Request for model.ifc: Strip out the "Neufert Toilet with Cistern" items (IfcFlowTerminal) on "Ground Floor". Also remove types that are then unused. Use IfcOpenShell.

First a look at what the model holds.

```python
import ifcopenshell
import ifcopenshell.util.element

model = ifcopenshell.open("model.ifc")
print(model.schema)
storey = next(s for s in model.by_type("IfcBuildingStorey") if s.Name == "Ground Floor")
terminals = [e for e in ifcopenshell.util.element.get_decomposition(storey) if e.is_a("IfcFlowTerminal")]
seen = {}
for e in terminals:
    element_type = ifcopenshell.util.element.get_type(e)
    name = element_type.Name if element_type not in (None, e) else None
    seen[name] = seen.get(name, 0) + 1
for name, count in sorted(seen.items(), key=str):
    print(count, "x", name)
```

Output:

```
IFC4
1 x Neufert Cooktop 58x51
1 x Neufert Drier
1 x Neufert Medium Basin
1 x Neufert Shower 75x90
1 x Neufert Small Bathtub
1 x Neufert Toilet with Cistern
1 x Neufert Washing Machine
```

```python
import ifcopenshell
import ifcopenshell.api.root
import ifcopenshell.util.element

model = ifcopenshell.open("model.ifc")

storey = next(s for s in model.by_type("IfcBuildingStorey") if s.Name == "Ground Floor")
terminals = [e for e in ifcopenshell.util.element.get_decomposition(storey) if e.is_a("IfcFlowTerminal")]
targets = [e for e in terminals if (t := ifcopenshell.util.element.get_type(e)) not in (None, e) and t.Name == "Neufert Toilet with Cistern"]
types = {ifcopenshell.util.element.get_type(e) for e in targets} - {None, *targets}

for e in targets:
    ifcopenshell.api.root.remove_product(model, product=e)
print(len(targets), "removed")

unused = [t for t in types if not ifcopenshell.util.element.get_types(t)]
for t in unused:
    ifcopenshell.api.root.remove_product(model, product=t)
print(len(unused), "unused types removed")

model.write("model_updated.ifc")
```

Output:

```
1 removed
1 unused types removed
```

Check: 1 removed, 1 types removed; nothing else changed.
